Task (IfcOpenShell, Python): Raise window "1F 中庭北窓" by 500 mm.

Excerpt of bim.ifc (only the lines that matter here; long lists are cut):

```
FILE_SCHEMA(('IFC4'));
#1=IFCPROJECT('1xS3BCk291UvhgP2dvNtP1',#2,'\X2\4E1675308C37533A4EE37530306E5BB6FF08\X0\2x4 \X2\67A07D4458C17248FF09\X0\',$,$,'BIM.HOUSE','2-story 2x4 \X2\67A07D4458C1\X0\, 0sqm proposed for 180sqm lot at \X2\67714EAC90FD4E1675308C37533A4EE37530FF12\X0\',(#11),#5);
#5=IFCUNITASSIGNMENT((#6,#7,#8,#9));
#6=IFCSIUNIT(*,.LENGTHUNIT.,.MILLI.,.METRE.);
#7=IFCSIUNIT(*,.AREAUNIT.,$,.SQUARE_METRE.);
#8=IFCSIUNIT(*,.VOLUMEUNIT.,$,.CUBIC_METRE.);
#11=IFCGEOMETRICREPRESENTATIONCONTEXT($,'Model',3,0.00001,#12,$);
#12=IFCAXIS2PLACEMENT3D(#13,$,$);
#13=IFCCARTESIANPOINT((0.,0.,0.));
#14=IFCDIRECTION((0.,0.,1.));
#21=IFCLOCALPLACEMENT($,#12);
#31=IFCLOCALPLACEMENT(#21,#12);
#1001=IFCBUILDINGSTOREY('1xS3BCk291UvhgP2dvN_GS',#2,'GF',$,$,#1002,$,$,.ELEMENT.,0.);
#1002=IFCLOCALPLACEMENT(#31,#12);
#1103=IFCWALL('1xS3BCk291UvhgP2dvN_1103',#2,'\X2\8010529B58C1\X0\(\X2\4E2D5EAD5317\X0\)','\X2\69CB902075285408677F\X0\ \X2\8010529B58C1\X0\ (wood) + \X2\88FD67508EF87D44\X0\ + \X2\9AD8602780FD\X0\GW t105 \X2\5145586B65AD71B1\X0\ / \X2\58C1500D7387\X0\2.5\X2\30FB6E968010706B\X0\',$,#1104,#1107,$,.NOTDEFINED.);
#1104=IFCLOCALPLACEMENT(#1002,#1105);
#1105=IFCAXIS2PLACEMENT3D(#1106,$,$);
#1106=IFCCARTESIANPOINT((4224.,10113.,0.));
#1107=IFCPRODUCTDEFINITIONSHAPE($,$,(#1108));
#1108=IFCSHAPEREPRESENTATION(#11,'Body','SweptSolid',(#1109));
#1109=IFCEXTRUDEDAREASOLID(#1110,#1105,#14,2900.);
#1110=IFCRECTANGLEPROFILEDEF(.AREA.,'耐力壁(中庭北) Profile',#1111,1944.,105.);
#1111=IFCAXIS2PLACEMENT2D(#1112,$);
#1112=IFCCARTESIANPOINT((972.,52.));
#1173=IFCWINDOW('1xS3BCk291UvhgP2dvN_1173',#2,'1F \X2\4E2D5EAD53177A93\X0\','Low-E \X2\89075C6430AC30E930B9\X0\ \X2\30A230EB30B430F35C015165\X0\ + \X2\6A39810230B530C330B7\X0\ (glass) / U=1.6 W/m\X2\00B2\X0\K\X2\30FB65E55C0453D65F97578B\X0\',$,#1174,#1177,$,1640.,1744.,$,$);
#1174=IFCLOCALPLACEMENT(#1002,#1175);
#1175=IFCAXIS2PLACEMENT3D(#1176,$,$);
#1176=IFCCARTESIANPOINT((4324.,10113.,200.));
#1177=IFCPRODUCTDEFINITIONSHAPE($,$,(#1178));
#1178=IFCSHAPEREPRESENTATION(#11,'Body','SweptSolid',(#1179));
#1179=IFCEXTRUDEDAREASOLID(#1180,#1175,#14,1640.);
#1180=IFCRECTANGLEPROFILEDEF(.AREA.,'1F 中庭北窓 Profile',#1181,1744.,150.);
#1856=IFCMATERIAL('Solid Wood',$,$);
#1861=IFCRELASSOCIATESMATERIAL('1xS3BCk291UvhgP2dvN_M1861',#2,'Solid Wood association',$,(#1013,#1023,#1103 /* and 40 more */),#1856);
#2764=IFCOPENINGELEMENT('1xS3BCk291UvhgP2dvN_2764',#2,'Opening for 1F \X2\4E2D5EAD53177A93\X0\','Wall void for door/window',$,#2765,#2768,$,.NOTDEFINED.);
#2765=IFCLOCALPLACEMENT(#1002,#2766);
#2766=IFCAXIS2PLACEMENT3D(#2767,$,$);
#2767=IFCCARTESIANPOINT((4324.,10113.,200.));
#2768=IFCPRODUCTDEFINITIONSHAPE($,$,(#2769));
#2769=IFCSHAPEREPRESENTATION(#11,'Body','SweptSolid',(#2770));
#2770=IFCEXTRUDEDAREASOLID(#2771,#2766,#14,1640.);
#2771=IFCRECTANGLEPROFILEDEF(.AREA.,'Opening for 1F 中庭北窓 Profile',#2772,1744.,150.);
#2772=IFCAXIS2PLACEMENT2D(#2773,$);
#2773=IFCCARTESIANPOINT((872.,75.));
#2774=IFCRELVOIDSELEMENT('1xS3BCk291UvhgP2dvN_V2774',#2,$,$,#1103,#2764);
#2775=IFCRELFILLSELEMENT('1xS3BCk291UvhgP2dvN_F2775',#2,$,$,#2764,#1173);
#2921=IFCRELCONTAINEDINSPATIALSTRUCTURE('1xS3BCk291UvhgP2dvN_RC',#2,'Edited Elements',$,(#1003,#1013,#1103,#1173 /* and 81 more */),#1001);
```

```python
import numpy as np
import ifcopenshell
import ifcopenshell.api.geometry
import ifcopenshell.util.placement
import ifcopenshell.util.unit

model = ifcopenshell.open("bim.ifc")
unit_scale = ifcopenshell.util.unit.calculate_unit_scale(model)

window = model.by_guid("1xS3BCk291UvhgP2dvN_1173")
opening = window.FillsVoids[0].RelatingOpeningElement
dz = 500.0

shift = np.array([0.0, 0.0, dz])
# The window is not placed relative to its opening, so move both.
for product in (opening, window):
    matrix = ifcopenshell.util.placement.get_local_placement(product.ObjectPlacement)
    matrix[:3, 3] += shift
    ifcopenshell.api.geometry.edit_object_placement(model, product=product, matrix=matrix, is_si=False)

print(f"moved by {dz * unit_scale:+.3f} m")

model.write("bim-out.ifc")
```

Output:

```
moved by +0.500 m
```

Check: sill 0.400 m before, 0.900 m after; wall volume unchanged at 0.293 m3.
